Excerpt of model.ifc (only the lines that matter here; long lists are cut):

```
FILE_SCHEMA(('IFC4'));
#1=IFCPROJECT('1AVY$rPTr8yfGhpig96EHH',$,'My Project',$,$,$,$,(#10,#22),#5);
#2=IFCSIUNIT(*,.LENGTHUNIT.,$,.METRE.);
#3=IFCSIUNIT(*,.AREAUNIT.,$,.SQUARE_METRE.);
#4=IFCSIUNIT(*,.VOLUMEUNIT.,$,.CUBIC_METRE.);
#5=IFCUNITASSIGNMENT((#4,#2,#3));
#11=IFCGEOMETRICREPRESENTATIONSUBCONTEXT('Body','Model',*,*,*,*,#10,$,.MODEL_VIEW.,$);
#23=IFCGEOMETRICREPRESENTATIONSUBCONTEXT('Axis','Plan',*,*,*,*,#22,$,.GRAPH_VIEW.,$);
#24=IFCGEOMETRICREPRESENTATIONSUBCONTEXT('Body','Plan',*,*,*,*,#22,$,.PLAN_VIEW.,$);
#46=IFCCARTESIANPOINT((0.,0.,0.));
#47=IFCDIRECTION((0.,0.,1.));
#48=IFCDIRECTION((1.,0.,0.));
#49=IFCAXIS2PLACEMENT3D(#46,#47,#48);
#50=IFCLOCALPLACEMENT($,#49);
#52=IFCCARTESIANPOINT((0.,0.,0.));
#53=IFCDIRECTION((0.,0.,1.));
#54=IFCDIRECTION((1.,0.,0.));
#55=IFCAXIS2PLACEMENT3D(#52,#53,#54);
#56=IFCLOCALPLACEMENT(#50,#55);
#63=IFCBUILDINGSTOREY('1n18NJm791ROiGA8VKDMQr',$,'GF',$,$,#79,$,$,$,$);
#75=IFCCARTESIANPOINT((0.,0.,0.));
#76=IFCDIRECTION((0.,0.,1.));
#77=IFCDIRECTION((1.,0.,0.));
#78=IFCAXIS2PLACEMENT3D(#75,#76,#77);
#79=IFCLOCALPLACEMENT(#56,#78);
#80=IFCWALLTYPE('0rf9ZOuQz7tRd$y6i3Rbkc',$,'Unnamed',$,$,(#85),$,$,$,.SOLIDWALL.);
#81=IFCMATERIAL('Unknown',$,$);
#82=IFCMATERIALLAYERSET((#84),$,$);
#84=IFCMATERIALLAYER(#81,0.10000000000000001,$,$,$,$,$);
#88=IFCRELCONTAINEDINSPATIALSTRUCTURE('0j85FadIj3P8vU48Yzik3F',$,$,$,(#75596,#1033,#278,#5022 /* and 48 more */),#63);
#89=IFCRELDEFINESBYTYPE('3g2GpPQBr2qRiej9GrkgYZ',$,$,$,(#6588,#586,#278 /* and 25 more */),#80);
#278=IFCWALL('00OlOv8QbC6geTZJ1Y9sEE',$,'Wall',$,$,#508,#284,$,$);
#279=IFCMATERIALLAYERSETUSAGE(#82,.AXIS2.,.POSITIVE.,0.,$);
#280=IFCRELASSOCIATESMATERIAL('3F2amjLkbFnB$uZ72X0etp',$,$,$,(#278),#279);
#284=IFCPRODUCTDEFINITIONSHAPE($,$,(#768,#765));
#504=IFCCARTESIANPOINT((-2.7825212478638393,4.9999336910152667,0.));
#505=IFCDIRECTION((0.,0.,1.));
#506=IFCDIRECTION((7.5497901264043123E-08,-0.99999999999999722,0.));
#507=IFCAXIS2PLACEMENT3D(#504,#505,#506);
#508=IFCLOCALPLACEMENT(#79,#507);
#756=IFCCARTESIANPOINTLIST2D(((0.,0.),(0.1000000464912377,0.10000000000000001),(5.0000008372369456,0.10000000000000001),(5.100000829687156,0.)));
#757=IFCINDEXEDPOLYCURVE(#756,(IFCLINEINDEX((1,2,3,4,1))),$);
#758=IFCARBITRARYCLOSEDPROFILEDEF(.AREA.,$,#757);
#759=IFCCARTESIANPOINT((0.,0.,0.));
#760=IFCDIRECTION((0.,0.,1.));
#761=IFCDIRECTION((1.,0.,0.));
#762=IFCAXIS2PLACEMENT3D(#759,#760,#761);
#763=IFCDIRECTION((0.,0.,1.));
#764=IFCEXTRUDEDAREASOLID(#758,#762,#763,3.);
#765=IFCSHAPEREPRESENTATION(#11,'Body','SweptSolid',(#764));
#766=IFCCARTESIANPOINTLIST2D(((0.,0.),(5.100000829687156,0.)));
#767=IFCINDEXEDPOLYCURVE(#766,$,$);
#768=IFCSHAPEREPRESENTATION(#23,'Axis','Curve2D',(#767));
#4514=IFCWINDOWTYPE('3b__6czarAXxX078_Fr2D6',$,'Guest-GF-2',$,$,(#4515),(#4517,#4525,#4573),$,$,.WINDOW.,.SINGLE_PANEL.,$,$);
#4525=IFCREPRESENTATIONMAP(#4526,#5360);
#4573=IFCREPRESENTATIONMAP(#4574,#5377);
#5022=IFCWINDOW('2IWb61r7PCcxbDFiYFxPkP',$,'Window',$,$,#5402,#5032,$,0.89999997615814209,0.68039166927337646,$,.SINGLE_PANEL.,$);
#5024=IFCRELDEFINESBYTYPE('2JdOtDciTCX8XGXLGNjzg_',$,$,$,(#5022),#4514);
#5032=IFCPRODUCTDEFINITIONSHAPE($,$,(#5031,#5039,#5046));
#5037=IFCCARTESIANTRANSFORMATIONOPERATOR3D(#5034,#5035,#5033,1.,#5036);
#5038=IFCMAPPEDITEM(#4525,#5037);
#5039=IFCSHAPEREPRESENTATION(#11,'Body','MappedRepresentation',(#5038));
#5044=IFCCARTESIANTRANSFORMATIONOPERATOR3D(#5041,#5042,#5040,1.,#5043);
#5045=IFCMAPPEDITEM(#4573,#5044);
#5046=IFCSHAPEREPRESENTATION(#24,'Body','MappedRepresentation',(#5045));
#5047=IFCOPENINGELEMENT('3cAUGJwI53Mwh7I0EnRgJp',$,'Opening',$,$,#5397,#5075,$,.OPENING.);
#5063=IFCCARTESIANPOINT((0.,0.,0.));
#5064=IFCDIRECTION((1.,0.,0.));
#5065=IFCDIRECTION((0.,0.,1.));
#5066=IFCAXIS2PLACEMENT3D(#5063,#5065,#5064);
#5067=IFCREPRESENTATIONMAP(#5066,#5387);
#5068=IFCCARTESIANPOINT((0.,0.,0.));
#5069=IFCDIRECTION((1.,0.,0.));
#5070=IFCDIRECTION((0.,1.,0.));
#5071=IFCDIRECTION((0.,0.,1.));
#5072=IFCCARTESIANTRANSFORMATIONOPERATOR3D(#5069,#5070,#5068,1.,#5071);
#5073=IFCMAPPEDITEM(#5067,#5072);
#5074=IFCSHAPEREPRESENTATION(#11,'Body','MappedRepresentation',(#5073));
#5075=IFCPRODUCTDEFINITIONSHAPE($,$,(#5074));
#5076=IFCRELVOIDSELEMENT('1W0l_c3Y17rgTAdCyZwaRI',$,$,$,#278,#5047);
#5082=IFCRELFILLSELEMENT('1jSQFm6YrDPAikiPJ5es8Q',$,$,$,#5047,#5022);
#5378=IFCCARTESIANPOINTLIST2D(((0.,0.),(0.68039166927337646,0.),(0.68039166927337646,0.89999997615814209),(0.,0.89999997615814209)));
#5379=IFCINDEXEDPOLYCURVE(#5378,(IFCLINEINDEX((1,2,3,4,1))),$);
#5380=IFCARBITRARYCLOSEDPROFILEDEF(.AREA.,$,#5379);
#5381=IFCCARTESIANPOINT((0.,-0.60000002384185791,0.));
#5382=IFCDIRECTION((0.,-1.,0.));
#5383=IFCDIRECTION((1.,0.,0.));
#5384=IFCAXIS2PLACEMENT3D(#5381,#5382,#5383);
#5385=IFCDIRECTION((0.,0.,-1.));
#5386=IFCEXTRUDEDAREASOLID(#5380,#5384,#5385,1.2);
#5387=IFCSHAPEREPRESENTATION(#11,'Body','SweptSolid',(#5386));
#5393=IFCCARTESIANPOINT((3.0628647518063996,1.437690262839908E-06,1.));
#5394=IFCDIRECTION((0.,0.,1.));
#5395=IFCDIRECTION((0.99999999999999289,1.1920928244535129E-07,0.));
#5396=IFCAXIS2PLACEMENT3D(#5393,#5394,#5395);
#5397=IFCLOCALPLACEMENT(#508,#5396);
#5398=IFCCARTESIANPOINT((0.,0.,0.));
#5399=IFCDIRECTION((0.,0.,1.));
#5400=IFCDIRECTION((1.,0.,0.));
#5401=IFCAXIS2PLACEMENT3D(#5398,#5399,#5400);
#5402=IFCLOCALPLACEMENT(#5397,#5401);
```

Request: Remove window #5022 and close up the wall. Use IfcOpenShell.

```python
import ifcopenshell
import ifcopenshell.api.feature
import ifcopenshell.api.root
import ifcopenshell.geom
import ifcopenshell.util.shape

model = ifcopenshell.open("model.ifc")
settings = ifcopenshell.geom.settings()


def volume(element):
    """Net volume in cubic metres, openings subtracted."""
    shape = ifcopenshell.geom.create_shape(settings, element)
    return ifcopenshell.util.shape.get_volume(shape.geometry)


window = model.by_guid("2IWb61r7PCcxbDFiYFxPkP")
opening = window.FillsVoids[0].RelatingOpeningElement
wall = opening.VoidsElements[0].RelatingBuildingElement
before = volume(wall)

ifcopenshell.api.root.remove_product(model, product=window)
ifcopenshell.api.feature.remove_feature(model, feature=opening)

after = volume(wall)

print(f"wall volume {before:.3f} -> {after:.3f} m3")

model.write("model_v2.ifc")
```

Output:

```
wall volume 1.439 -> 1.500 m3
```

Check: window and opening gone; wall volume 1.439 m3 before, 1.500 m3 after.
